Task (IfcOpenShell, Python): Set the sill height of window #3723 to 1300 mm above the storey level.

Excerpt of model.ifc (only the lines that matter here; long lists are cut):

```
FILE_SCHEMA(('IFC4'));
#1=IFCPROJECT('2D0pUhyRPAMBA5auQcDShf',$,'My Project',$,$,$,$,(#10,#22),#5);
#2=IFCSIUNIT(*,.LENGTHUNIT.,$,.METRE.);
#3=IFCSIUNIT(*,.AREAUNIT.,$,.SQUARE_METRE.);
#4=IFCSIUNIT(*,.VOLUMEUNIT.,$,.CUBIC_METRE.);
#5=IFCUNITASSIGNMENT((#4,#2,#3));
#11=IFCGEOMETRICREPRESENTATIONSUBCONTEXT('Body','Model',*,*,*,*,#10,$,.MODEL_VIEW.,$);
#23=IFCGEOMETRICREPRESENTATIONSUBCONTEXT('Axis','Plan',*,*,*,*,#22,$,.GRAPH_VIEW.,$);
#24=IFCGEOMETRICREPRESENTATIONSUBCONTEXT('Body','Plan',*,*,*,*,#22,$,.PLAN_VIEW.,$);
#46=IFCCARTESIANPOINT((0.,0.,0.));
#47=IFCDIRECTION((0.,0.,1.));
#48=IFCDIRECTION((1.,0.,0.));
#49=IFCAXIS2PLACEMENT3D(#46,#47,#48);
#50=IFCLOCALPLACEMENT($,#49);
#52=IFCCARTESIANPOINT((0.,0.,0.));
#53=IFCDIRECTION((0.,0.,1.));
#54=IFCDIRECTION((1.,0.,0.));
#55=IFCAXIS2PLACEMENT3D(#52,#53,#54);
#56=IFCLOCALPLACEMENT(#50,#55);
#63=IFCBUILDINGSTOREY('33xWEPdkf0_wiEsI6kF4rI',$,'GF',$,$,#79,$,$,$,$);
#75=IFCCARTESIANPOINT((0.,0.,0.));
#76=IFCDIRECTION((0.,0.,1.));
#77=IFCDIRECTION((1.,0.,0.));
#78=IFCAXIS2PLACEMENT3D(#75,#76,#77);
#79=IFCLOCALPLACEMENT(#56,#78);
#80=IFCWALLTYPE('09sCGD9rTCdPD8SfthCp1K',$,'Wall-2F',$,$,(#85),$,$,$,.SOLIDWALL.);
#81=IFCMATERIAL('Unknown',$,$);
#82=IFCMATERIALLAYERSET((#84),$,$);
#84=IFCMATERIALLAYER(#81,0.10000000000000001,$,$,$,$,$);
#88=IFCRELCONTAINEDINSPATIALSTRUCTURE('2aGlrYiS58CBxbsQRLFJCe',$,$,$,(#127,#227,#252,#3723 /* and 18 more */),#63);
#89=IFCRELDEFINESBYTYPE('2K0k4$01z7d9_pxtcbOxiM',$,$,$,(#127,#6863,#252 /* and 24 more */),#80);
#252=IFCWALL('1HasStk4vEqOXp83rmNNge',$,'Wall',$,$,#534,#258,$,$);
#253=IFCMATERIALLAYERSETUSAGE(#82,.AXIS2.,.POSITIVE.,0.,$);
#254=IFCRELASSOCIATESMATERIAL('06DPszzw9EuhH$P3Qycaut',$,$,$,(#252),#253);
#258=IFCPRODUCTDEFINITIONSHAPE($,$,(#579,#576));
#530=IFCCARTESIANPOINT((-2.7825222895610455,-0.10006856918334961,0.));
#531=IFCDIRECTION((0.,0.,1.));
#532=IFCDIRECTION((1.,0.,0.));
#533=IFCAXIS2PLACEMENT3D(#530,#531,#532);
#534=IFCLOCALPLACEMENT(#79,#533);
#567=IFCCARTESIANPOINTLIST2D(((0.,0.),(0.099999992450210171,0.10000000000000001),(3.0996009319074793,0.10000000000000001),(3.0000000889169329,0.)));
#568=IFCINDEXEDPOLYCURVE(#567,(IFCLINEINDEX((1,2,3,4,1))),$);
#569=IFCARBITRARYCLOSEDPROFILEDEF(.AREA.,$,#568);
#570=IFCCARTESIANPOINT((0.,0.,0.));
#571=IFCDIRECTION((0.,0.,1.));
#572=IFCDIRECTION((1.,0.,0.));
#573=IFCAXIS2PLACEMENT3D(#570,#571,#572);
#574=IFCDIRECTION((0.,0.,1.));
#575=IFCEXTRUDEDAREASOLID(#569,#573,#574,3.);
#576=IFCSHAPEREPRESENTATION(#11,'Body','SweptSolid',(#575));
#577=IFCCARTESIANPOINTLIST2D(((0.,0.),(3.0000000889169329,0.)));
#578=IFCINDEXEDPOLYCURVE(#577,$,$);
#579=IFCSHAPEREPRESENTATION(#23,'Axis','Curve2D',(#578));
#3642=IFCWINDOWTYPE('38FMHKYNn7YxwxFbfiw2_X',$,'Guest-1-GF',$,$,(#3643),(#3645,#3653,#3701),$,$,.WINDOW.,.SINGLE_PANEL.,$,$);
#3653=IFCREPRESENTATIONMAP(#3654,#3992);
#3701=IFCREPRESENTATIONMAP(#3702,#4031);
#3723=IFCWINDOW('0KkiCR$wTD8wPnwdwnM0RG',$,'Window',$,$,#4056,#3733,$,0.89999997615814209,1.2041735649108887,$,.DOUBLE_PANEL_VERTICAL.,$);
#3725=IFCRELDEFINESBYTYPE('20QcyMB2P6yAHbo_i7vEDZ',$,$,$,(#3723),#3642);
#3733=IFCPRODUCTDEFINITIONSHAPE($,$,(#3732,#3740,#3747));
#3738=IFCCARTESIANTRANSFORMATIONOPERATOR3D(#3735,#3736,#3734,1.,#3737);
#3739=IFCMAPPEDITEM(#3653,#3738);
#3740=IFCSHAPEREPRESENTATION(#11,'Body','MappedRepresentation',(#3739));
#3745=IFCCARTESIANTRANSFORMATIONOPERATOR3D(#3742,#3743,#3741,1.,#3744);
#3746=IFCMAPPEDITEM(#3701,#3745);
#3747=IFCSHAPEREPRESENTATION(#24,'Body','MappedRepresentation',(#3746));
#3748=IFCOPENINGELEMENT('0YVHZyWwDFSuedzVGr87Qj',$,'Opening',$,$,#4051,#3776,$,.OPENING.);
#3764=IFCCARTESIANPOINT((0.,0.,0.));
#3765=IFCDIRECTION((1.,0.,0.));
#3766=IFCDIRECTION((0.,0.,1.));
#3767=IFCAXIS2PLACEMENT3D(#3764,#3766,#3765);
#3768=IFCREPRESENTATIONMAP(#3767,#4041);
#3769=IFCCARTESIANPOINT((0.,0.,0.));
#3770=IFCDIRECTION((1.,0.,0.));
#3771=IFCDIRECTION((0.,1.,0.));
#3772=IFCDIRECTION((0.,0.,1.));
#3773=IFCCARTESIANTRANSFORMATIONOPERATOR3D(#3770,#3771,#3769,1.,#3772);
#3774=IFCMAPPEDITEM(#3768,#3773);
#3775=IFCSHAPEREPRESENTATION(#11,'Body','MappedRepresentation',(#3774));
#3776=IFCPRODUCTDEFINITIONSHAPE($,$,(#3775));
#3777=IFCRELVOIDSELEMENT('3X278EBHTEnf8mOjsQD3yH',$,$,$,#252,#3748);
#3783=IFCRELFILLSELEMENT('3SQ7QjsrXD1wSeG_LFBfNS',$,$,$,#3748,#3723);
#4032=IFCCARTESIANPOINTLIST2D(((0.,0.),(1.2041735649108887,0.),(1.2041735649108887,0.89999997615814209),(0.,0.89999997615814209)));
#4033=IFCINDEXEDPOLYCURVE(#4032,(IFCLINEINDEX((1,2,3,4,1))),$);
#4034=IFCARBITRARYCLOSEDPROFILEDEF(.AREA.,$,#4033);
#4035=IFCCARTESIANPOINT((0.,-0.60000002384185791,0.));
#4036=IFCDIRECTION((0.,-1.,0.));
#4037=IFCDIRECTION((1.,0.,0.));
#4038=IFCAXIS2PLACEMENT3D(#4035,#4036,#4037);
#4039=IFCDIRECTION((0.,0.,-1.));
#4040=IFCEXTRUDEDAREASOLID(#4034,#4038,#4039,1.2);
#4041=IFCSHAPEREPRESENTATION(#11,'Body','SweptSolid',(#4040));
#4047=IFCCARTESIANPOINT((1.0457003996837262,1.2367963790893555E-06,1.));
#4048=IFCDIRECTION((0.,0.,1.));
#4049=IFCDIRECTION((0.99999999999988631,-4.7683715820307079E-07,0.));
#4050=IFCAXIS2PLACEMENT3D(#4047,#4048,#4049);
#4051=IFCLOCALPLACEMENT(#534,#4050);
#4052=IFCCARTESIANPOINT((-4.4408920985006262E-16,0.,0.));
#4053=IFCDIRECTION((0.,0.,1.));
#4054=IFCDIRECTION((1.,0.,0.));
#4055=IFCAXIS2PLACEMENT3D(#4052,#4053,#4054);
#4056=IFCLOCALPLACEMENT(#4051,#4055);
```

```python
import numpy as np
import ifcopenshell
import ifcopenshell.api.geometry
import ifcopenshell.geom
import ifcopenshell.util.element
import ifcopenshell.util.placement
import ifcopenshell.util.shape
import ifcopenshell.util.unit

model = ifcopenshell.open("model.ifc")
unit_scale = ifcopenshell.util.unit.calculate_unit_scale(model)

window = model.by_guid("0KkiCR$wTD8wPnwdwnM0RG")
opening = window.FillsVoids[0].RelatingOpeningElement
storey = ifcopenshell.util.element.get_container(window, ifc_class="IfcBuildingStorey")
level = ifcopenshell.util.placement.get_local_placement(storey.ObjectPlacement)[2, 3]

# The opening's origin need not be at the sill, so measure its lowest point.
shape = ifcopenshell.geom.create_shape(ifcopenshell.geom.settings(), opening)
bottom = ifcopenshell.util.shape.get_shape_bottom_elevation(shape, shape.geometry) / unit_scale
dz = level + 1.3 / unit_scale - bottom

shift = np.array([0.0, 0.0, dz])
# The window is placed relative to its opening, so it follows when the opening moves.
matrix = ifcopenshell.util.placement.get_local_placement(opening.ObjectPlacement)
matrix[:3, 3] += shift
ifcopenshell.api.geometry.edit_object_placement(
    model, product=opening, matrix=matrix, is_si=False, should_transform_children=True
)

print(f"moved by {dz * unit_scale:+.3f} m")

model.write("model-out.ifc")
```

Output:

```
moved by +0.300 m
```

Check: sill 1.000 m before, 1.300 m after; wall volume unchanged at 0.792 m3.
